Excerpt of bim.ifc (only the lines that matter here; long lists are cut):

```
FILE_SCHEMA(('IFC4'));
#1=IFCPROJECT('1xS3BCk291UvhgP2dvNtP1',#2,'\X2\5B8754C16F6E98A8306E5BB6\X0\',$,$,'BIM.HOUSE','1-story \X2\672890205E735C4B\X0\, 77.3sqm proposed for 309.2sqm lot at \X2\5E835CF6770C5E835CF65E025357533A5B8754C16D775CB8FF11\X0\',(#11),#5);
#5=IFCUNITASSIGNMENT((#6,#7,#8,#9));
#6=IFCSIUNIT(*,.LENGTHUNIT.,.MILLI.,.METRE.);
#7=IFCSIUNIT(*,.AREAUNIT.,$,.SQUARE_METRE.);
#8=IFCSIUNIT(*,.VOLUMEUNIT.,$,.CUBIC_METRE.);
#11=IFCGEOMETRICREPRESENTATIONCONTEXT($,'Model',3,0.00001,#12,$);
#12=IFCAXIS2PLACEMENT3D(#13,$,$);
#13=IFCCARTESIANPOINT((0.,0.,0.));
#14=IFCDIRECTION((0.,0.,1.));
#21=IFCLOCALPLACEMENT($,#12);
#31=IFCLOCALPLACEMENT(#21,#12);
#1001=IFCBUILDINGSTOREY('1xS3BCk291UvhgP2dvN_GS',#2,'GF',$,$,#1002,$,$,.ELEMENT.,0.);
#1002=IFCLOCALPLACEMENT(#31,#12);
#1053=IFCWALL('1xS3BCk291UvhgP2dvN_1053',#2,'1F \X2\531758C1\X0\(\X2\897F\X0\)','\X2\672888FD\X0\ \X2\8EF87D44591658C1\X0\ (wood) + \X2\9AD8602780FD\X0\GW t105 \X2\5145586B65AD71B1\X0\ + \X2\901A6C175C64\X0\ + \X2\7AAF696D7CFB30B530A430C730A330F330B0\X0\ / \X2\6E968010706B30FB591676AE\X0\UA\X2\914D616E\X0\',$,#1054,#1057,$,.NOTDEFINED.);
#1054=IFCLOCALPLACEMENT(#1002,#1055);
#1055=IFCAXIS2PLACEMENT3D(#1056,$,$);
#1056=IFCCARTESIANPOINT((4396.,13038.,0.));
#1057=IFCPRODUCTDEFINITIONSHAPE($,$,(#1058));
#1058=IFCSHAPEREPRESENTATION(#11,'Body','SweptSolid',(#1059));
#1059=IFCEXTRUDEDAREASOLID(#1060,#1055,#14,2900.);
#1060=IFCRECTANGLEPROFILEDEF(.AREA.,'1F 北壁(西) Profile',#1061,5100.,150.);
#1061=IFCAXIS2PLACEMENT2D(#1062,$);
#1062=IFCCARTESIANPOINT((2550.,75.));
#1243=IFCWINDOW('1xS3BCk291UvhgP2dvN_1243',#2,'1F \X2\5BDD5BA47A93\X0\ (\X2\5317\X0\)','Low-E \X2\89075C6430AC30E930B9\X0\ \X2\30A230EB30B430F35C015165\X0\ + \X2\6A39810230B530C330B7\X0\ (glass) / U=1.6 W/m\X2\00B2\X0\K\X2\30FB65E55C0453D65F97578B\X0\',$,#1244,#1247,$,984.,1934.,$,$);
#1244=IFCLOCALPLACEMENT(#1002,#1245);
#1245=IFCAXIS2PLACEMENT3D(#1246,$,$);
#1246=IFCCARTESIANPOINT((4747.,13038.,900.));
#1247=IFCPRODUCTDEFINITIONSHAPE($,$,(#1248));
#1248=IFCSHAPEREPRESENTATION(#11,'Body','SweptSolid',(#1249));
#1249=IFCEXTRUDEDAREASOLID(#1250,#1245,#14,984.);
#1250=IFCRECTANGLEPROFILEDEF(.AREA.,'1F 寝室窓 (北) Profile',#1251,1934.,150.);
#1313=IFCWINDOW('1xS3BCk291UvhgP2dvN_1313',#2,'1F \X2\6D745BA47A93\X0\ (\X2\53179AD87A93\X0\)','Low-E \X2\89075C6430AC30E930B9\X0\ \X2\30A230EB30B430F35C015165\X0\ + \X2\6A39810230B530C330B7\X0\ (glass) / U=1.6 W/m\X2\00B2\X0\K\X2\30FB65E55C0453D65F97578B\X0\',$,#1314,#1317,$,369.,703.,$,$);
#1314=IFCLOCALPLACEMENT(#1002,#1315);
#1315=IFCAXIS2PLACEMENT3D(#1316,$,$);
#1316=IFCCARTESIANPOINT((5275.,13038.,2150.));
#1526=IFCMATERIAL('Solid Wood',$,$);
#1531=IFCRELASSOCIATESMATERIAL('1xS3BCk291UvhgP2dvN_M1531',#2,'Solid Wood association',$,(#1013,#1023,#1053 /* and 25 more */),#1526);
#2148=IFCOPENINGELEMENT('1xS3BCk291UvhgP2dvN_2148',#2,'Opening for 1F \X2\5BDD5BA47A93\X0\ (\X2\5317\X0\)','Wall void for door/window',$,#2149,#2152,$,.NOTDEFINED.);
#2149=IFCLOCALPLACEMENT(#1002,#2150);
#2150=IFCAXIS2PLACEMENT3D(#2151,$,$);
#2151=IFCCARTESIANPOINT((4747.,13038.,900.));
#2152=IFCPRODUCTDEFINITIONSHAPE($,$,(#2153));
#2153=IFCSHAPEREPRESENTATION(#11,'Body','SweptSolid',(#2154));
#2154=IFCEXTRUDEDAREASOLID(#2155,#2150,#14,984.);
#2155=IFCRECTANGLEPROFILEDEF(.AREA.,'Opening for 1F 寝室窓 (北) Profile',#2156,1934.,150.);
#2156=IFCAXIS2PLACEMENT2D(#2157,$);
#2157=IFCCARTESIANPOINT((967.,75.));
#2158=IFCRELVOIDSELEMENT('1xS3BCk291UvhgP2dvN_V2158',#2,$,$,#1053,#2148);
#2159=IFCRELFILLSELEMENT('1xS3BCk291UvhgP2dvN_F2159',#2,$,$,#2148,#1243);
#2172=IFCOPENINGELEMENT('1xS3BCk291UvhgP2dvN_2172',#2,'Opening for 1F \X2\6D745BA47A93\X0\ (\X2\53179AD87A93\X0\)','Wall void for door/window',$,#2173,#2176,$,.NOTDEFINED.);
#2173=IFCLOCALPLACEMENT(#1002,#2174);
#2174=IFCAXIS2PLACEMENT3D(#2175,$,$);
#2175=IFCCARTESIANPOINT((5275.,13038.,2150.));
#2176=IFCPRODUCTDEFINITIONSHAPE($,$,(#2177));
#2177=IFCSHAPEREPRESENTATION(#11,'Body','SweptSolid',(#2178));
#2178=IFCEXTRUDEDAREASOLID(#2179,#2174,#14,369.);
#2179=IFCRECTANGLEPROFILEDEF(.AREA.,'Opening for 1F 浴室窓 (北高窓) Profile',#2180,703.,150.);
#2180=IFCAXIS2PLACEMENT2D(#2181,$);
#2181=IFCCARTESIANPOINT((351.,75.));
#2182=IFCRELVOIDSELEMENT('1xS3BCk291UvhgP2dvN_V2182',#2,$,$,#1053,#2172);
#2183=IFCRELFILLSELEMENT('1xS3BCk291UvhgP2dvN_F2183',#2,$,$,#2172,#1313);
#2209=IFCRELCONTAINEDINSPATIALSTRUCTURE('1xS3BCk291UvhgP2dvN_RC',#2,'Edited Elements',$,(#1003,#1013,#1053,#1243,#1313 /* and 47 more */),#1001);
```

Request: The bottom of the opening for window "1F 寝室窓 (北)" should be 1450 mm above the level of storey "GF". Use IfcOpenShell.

```python
import numpy as np
import ifcopenshell
import ifcopenshell.api.geometry
import ifcopenshell.geom
import ifcopenshell.util.element
import ifcopenshell.util.placement
import ifcopenshell.util.shape
import ifcopenshell.util.unit

model = ifcopenshell.open("bim.ifc")
unit_scale = ifcopenshell.util.unit.calculate_unit_scale(model)

window = model.by_guid("1xS3BCk291UvhgP2dvN_1243")
opening = window.FillsVoids[0].RelatingOpeningElement
storey = ifcopenshell.util.element.get_container(window, ifc_class="IfcBuildingStorey")
level = ifcopenshell.util.placement.get_local_placement(storey.ObjectPlacement)[2, 3]

# The opening's origin need not be at the sill, so measure its lowest point.
shape = ifcopenshell.geom.create_shape(ifcopenshell.geom.settings(), opening)
bottom = ifcopenshell.util.shape.get_shape_bottom_elevation(shape, shape.geometry) / unit_scale
dz = level + 1.45 / unit_scale - bottom

shift = np.array([0.0, 0.0, dz])
# The window is not placed relative to its opening, so move both.
for product in (opening, window):
    matrix = ifcopenshell.util.placement.get_local_placement(product.ObjectPlacement)
    matrix[:3, 3] += shift
    ifcopenshell.api.geometry.edit_object_placement(model, product=product, matrix=matrix, is_si=False)

print(f"moved by {dz * unit_scale:+.3f} m")

model.write("bim_updated.ifc")
```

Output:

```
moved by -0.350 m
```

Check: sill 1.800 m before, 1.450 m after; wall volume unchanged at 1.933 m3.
